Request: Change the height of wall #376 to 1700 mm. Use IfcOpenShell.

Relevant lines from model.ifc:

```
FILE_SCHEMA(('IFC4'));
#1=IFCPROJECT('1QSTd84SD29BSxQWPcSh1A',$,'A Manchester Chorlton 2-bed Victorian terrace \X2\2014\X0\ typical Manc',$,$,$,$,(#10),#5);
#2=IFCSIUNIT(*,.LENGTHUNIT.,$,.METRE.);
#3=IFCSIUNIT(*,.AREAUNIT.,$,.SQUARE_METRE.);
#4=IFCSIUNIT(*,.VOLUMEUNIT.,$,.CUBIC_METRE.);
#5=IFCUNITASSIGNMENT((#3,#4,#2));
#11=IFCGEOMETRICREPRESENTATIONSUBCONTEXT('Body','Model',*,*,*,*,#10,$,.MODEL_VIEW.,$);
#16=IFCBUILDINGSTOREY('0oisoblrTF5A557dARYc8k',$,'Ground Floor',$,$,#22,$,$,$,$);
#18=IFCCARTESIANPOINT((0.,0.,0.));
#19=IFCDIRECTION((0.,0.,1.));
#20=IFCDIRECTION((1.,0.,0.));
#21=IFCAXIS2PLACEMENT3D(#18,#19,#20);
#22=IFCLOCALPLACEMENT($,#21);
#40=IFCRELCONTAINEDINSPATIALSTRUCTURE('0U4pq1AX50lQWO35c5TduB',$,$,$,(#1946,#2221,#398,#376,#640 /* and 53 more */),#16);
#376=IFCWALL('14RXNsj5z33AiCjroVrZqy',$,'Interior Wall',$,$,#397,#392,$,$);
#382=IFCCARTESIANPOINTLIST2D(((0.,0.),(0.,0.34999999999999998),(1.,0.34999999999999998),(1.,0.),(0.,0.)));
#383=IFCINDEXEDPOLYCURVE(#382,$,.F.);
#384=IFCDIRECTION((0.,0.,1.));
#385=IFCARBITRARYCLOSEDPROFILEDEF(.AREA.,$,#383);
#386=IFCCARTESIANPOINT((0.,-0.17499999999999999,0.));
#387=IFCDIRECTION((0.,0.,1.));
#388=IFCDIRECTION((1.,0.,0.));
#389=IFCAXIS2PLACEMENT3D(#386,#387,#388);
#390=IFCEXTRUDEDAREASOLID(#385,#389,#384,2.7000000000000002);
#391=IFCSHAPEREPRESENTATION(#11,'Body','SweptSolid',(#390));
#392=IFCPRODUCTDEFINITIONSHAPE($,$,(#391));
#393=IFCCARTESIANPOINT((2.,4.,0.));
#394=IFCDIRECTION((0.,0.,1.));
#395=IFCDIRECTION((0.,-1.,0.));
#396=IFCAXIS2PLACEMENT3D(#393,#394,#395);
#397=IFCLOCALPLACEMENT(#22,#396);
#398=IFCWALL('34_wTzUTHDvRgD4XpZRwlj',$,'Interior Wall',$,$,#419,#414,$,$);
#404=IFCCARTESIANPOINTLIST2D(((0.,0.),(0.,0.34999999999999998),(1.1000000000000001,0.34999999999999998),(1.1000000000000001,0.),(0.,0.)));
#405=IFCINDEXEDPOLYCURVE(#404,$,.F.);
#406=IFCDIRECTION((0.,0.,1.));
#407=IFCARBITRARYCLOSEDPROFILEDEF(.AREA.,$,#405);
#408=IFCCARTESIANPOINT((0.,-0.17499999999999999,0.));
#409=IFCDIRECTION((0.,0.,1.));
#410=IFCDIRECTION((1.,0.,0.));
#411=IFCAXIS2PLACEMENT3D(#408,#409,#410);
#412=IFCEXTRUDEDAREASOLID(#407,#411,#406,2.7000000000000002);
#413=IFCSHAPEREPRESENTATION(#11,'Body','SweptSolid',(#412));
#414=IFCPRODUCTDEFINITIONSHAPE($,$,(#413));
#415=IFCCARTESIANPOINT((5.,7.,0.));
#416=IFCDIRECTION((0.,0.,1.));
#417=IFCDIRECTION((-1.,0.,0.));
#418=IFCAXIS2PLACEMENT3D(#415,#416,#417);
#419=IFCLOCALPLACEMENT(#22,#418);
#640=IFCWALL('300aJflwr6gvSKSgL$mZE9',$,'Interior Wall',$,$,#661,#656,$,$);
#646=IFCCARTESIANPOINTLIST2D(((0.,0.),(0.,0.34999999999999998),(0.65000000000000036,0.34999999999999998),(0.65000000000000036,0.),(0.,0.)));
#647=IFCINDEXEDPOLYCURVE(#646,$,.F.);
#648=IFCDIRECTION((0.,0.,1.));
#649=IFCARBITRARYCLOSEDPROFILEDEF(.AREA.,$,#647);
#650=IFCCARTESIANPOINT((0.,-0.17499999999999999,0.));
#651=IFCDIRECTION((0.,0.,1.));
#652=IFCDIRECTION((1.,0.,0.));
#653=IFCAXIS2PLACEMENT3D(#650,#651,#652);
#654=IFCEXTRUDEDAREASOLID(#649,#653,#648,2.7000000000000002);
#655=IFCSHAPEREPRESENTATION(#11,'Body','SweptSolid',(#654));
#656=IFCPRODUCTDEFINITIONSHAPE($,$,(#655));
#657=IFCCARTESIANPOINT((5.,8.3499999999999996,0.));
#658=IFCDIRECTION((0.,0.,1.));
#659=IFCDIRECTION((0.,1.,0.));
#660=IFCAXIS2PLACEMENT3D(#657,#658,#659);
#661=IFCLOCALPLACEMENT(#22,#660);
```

```python
import ifcopenshell
import ifcopenshell.geom
import ifcopenshell.util.representation
import ifcopenshell.util.shape

model = ifcopenshell.open("model.ifc")
settings = ifcopenshell.geom.settings()


def volume(element):
    """Net volume in cubic metres, openings subtracted."""
    shape = ifcopenshell.geom.create_shape(settings, element)
    return ifcopenshell.util.shape.get_volume(shape.geometry)


wall = model.by_id(376)
before = volume(wall)

body = ifcopenshell.util.representation.get_representation(wall, "Model", "Body")
solid = body.Items[0]
old_height = solid.Depth
solid.Depth = 1.7
after = volume(wall)

print(f"height {old_height:g} -> {solid.Depth:g}, volume {before:.3f} -> {after:.3f} m3")

model.write("model_v2.ifc")
```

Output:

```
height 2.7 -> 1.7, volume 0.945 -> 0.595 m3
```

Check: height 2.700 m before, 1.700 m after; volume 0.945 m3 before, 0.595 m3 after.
